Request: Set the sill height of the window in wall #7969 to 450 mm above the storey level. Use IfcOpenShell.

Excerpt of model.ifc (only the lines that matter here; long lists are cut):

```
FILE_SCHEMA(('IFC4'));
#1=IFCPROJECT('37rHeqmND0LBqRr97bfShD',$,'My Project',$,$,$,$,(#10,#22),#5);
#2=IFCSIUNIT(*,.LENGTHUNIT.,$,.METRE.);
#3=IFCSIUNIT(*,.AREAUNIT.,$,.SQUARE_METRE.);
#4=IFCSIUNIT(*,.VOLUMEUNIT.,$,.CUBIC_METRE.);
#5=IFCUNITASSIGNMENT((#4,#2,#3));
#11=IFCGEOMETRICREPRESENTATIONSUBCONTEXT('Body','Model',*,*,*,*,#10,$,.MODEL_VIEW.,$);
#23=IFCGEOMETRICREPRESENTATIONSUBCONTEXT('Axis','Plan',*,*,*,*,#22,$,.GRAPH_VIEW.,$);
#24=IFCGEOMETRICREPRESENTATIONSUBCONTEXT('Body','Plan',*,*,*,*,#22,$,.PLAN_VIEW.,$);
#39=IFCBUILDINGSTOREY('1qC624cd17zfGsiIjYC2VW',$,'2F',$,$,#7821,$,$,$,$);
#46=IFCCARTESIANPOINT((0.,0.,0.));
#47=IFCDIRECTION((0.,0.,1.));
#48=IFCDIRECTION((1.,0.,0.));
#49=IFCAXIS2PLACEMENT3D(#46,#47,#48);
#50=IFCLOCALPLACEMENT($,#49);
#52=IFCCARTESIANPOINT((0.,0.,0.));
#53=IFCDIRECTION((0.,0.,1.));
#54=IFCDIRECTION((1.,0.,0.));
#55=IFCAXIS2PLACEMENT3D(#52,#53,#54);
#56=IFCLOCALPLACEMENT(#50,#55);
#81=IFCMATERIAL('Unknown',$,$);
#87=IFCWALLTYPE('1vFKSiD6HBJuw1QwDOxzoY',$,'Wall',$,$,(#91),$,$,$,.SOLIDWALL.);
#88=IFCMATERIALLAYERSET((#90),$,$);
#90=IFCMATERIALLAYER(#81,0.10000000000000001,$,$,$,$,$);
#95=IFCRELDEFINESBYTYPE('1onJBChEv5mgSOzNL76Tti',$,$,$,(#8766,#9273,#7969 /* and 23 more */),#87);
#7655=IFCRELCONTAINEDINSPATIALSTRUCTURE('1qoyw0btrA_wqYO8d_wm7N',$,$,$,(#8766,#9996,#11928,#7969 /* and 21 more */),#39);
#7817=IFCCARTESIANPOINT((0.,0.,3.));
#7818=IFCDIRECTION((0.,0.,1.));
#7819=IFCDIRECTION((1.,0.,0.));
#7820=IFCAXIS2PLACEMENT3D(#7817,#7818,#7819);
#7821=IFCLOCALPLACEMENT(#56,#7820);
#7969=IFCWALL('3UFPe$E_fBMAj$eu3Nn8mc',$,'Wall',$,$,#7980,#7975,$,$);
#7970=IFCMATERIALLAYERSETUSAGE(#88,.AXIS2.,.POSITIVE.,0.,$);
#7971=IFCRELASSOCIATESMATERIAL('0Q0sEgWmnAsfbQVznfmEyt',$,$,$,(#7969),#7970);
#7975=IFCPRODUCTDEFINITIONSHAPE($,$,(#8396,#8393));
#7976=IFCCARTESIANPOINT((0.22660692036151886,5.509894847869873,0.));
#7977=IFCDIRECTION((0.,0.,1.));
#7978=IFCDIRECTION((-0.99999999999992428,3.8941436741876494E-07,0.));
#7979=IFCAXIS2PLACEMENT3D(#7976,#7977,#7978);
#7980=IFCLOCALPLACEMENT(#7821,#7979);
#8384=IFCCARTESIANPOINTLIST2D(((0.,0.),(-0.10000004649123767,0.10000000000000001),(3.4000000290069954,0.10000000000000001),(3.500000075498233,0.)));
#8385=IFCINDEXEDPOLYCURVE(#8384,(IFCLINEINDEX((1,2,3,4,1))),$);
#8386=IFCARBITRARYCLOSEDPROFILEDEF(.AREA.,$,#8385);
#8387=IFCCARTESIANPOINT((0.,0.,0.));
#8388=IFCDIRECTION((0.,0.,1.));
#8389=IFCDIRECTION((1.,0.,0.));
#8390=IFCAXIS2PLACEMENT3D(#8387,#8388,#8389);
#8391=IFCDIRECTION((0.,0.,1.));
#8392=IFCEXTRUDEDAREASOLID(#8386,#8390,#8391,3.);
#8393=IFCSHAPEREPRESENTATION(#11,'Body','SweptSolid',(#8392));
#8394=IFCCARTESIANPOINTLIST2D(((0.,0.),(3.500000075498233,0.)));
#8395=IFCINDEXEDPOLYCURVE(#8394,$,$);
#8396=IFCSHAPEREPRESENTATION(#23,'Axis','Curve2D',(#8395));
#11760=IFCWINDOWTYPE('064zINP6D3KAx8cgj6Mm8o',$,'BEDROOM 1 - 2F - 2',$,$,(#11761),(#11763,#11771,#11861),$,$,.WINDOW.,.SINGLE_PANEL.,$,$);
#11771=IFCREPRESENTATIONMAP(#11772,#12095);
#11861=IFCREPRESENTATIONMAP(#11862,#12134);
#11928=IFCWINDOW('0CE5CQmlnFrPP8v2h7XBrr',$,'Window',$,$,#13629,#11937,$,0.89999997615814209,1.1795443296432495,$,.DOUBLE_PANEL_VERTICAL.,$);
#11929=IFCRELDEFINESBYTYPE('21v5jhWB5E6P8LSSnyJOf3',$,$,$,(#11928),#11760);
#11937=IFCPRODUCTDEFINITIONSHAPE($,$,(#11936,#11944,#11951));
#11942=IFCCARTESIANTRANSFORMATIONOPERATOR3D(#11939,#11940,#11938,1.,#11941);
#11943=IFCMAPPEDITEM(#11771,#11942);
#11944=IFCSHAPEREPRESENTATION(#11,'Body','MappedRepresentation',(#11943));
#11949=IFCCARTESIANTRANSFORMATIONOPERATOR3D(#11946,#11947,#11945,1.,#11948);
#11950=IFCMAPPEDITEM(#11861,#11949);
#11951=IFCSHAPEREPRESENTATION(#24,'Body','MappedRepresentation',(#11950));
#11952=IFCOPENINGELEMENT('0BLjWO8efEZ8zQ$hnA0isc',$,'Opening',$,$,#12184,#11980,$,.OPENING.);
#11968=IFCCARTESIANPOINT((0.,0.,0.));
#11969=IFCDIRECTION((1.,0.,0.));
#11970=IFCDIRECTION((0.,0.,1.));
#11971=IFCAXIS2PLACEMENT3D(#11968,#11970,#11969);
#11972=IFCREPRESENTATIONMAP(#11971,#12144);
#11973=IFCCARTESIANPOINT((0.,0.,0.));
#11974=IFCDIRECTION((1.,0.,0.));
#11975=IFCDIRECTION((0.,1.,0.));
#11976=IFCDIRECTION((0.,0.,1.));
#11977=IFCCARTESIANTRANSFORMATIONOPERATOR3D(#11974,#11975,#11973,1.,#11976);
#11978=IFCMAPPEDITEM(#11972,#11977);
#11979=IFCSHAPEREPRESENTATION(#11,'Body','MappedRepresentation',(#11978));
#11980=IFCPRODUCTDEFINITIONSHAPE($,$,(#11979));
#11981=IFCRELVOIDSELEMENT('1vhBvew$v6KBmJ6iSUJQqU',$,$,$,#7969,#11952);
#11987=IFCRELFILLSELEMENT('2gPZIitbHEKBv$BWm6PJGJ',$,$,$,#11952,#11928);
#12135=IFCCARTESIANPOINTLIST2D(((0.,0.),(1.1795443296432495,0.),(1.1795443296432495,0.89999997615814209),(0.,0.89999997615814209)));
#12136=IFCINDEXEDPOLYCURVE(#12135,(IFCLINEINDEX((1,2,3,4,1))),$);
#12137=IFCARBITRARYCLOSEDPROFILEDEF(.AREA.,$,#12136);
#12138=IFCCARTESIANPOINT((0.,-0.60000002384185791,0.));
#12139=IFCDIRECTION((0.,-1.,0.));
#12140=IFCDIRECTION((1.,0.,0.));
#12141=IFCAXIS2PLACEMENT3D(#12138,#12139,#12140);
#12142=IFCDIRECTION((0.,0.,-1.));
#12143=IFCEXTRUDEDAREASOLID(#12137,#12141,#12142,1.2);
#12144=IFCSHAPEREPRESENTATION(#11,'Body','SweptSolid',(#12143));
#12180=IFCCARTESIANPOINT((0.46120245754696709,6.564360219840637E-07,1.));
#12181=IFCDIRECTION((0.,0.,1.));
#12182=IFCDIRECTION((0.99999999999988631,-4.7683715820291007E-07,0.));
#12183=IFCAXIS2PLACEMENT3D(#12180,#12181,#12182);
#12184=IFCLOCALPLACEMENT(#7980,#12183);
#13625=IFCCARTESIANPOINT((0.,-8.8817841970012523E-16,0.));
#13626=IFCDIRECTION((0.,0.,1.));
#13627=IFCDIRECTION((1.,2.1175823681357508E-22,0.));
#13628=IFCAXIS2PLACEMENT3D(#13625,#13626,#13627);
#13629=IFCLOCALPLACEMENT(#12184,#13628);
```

```python
import numpy as np
import ifcopenshell
import ifcopenshell.api.geometry
import ifcopenshell.geom
import ifcopenshell.util.element
import ifcopenshell.util.placement
import ifcopenshell.util.shape
import ifcopenshell.util.unit

model = ifcopenshell.open("model.ifc")
unit_scale = ifcopenshell.util.unit.calculate_unit_scale(model)

window = model.by_guid("0CE5CQmlnFrPP8v2h7XBrr")
opening = window.FillsVoids[0].RelatingOpeningElement
storey = ifcopenshell.util.element.get_container(window, ifc_class="IfcBuildingStorey")
level = ifcopenshell.util.placement.get_local_placement(storey.ObjectPlacement)[2, 3]

# The opening's origin need not be at the sill, so measure its lowest point.
shape = ifcopenshell.geom.create_shape(ifcopenshell.geom.settings(), opening)
bottom = ifcopenshell.util.shape.get_shape_bottom_elevation(shape, shape.geometry) / unit_scale
dz = level + 0.45 / unit_scale - bottom

shift = np.array([0.0, 0.0, dz])
# The window is placed relative to its opening, so it follows when the opening moves.
matrix = ifcopenshell.util.placement.get_local_placement(opening.ObjectPlacement)
matrix[:3, 3] += shift
ifcopenshell.api.geometry.edit_object_placement(
    model, product=opening, matrix=matrix, is_si=False, should_transform_children=True
)

print(f"moved by {dz * unit_scale:+.3f} m")

model.write("model-out.ifc")
```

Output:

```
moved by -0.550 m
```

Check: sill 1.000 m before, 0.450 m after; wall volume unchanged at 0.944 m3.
